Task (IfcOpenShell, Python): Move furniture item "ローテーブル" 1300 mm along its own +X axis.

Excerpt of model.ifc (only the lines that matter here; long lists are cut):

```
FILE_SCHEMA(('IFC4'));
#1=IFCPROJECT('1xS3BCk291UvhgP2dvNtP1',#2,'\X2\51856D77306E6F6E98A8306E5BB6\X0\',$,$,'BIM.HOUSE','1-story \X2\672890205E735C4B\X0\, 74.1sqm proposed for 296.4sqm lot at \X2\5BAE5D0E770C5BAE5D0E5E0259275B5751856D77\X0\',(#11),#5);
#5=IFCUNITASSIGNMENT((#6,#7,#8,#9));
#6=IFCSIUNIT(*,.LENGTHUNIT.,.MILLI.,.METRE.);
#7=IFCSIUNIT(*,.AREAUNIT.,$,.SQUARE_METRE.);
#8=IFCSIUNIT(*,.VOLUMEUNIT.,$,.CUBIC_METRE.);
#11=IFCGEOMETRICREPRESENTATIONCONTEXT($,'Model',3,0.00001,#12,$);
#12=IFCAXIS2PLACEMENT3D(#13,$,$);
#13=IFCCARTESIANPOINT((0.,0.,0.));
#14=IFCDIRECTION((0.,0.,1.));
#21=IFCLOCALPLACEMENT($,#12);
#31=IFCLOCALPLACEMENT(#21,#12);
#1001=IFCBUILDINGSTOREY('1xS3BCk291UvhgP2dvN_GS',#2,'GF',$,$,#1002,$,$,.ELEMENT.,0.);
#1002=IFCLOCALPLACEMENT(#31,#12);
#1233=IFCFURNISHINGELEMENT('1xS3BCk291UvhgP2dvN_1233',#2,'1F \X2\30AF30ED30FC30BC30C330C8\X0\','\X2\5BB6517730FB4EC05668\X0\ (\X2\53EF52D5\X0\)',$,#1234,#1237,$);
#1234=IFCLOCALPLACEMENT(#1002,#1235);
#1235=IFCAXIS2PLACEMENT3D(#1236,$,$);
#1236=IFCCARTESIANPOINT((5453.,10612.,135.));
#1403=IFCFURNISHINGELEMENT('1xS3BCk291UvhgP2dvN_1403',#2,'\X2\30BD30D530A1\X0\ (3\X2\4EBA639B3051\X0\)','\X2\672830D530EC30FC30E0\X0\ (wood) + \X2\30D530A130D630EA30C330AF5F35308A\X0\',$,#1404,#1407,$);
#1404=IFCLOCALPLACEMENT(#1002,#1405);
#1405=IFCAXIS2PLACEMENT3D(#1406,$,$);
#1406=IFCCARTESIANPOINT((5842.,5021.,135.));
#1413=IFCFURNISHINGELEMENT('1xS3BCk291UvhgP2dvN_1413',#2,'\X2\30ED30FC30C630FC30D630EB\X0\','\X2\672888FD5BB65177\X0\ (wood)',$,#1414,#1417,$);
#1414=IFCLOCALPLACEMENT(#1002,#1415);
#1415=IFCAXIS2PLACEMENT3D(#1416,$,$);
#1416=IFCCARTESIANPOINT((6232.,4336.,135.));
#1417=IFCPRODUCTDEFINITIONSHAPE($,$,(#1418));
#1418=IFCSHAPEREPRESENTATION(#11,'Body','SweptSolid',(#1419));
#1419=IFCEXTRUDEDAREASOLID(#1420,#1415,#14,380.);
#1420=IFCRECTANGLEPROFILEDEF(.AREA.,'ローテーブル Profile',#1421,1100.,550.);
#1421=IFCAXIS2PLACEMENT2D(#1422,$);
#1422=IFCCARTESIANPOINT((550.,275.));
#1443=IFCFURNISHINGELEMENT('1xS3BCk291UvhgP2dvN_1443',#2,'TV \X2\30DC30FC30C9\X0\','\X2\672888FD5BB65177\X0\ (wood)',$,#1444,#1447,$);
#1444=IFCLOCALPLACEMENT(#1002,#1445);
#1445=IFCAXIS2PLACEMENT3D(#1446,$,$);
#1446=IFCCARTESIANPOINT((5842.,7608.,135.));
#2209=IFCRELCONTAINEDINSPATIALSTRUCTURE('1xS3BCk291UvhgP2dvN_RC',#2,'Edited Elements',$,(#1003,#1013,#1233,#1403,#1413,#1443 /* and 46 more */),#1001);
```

```python
import ifcopenshell
import ifcopenshell.api.geometry
import ifcopenshell.util.placement

model = ifcopenshell.open("model.ifc")

item = model.by_guid("1xS3BCk291UvhgP2dvN_1413")
matrix = ifcopenshell.util.placement.get_local_placement(item.ObjectPlacement)
matrix[:3, 3] += matrix[:3, 0] * 1300.0
ifcopenshell.api.geometry.edit_object_placement(model, product=item, matrix=matrix, is_si=False)

print(ifcopenshell.util.placement.get_local_placement(item.ObjectPlacement).round(3) + 0.0)

model.write("model_v2.ifc")
```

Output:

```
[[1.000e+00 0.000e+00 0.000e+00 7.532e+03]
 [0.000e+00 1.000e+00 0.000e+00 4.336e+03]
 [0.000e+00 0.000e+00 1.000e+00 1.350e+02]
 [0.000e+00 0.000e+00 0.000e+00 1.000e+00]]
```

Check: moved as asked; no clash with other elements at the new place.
